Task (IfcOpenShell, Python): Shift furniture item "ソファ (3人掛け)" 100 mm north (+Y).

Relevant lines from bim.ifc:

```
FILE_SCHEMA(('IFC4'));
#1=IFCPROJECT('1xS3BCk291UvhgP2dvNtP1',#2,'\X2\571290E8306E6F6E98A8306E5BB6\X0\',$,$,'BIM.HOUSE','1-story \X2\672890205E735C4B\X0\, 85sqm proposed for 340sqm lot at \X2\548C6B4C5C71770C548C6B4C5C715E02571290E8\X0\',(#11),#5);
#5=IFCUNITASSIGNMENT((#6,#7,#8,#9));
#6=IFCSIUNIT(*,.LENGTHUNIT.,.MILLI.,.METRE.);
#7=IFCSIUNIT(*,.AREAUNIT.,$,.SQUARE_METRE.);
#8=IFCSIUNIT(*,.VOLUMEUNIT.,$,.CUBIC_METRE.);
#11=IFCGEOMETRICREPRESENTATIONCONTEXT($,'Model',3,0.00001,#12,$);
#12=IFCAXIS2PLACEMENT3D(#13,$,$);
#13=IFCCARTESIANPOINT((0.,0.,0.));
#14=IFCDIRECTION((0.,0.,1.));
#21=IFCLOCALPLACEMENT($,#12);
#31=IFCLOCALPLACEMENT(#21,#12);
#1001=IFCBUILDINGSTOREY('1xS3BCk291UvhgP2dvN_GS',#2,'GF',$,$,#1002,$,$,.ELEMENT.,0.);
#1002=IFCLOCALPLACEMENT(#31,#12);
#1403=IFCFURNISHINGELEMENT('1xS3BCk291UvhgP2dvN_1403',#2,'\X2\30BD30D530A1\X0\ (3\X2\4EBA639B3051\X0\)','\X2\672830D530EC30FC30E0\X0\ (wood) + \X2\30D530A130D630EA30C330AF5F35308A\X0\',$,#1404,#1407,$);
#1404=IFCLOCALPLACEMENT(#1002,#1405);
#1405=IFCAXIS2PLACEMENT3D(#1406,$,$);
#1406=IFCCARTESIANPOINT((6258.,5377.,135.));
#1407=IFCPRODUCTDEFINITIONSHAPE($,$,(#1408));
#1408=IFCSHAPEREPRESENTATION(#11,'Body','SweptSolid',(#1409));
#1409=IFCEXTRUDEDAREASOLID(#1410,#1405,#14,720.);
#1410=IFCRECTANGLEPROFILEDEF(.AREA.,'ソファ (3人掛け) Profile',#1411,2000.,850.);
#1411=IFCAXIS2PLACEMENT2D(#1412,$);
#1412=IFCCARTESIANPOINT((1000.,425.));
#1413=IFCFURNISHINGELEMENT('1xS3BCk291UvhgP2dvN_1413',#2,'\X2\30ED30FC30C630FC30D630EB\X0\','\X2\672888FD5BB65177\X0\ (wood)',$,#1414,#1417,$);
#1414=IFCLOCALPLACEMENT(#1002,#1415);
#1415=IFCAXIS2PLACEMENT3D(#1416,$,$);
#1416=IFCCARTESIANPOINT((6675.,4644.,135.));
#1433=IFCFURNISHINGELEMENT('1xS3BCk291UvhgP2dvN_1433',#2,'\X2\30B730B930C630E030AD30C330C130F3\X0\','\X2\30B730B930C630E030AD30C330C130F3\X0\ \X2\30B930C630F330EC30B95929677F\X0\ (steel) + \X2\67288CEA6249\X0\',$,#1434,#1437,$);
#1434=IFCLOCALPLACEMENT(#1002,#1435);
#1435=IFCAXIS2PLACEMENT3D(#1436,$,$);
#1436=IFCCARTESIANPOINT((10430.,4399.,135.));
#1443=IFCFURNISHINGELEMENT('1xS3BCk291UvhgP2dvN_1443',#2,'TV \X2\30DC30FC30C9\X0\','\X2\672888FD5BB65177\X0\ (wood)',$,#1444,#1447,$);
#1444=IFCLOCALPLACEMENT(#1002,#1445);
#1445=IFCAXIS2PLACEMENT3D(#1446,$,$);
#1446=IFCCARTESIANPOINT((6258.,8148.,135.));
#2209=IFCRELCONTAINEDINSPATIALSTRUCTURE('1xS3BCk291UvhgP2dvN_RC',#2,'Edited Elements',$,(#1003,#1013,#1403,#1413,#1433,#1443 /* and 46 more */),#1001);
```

```python
import ifcopenshell
import ifcopenshell.api.geometry
import ifcopenshell.util.placement

model = ifcopenshell.open("bim.ifc")

item = model.by_id(1403)
matrix = ifcopenshell.util.placement.get_local_placement(item.ObjectPlacement)
matrix[1, 3] += 100.0
ifcopenshell.api.geometry.edit_object_placement(model, product=item, matrix=matrix, is_si=False)

print(ifcopenshell.util.placement.get_local_placement(item.ObjectPlacement).round(3) + 0.0)

model.write("bim_updated.ifc")
```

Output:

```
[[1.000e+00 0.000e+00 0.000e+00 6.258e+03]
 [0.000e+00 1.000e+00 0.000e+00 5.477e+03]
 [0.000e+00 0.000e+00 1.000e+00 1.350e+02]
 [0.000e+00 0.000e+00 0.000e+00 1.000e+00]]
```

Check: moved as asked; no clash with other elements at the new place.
